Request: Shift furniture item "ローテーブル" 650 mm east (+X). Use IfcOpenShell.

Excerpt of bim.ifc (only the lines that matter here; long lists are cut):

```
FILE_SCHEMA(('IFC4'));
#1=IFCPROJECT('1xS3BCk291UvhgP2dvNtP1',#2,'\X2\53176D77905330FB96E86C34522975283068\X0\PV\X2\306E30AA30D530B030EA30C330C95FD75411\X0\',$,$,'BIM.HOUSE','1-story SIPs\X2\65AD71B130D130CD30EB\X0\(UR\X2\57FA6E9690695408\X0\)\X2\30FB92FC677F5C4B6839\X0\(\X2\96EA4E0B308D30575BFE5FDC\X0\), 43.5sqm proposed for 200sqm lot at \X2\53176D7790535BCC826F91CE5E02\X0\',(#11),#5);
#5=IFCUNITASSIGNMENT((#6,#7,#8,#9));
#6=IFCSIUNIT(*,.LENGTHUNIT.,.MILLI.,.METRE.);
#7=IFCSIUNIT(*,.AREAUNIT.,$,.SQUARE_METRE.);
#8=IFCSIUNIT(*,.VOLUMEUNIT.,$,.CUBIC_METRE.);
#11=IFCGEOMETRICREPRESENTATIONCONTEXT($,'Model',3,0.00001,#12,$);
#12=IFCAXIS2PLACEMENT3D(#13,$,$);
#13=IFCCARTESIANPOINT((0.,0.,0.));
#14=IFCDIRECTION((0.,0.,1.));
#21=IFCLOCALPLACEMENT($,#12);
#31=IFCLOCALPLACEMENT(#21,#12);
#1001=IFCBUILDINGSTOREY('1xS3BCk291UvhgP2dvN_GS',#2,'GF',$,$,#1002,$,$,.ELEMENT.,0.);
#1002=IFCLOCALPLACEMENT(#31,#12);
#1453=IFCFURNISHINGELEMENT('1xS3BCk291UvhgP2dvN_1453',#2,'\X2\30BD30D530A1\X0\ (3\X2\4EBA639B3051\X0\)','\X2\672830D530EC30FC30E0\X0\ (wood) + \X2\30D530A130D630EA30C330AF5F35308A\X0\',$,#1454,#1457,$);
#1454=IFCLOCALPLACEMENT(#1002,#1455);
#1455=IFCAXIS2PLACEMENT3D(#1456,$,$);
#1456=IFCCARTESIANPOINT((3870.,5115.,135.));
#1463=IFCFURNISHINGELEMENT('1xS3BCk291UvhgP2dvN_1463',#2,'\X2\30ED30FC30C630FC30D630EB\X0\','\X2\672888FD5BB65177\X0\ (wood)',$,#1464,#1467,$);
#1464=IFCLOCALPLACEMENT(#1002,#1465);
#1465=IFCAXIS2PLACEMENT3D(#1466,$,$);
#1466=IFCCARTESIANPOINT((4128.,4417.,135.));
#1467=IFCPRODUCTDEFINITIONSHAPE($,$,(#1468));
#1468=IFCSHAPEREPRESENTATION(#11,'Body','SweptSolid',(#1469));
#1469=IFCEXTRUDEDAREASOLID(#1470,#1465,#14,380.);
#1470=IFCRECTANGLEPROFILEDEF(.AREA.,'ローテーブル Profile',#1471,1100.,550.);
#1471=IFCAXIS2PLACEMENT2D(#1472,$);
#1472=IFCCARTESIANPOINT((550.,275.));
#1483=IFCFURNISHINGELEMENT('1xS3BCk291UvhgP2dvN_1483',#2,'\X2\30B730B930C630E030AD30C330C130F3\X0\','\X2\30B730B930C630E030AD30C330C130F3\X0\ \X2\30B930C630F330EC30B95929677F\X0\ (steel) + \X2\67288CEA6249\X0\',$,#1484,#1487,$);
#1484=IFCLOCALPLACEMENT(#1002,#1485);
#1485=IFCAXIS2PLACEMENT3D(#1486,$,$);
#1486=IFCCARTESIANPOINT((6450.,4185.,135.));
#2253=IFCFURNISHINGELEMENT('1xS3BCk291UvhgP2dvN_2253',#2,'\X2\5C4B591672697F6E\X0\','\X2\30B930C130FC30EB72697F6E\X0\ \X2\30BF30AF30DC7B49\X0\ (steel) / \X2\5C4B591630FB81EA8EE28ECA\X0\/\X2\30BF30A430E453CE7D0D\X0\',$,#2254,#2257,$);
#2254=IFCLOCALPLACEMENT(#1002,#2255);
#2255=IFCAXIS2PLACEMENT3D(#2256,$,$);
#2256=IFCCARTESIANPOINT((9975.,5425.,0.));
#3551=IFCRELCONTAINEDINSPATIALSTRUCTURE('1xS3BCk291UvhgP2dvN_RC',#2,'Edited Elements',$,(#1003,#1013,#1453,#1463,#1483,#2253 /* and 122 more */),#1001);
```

```python
import ifcopenshell
import ifcopenshell.api.geometry
import ifcopenshell.util.placement
import ifcopenshell.util.unit

model = ifcopenshell.open("bim.ifc")
unit_scale = ifcopenshell.util.unit.calculate_unit_scale(model)

item = model.by_guid("1xS3BCk291UvhgP2dvN_1463")
matrix = ifcopenshell.util.placement.get_local_placement(item.ObjectPlacement)
matrix[0, 3] += 0.65 / unit_scale
ifcopenshell.api.geometry.edit_object_placement(model, product=item, matrix=matrix, is_si=False)

print(ifcopenshell.util.placement.get_local_placement(item.ObjectPlacement).round(3) + 0.0)

model.write("bim_v2.ifc")
```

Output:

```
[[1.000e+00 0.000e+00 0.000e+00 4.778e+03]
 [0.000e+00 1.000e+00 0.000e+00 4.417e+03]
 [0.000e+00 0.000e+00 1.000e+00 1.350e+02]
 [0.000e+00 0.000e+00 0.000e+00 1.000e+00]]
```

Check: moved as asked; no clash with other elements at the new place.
